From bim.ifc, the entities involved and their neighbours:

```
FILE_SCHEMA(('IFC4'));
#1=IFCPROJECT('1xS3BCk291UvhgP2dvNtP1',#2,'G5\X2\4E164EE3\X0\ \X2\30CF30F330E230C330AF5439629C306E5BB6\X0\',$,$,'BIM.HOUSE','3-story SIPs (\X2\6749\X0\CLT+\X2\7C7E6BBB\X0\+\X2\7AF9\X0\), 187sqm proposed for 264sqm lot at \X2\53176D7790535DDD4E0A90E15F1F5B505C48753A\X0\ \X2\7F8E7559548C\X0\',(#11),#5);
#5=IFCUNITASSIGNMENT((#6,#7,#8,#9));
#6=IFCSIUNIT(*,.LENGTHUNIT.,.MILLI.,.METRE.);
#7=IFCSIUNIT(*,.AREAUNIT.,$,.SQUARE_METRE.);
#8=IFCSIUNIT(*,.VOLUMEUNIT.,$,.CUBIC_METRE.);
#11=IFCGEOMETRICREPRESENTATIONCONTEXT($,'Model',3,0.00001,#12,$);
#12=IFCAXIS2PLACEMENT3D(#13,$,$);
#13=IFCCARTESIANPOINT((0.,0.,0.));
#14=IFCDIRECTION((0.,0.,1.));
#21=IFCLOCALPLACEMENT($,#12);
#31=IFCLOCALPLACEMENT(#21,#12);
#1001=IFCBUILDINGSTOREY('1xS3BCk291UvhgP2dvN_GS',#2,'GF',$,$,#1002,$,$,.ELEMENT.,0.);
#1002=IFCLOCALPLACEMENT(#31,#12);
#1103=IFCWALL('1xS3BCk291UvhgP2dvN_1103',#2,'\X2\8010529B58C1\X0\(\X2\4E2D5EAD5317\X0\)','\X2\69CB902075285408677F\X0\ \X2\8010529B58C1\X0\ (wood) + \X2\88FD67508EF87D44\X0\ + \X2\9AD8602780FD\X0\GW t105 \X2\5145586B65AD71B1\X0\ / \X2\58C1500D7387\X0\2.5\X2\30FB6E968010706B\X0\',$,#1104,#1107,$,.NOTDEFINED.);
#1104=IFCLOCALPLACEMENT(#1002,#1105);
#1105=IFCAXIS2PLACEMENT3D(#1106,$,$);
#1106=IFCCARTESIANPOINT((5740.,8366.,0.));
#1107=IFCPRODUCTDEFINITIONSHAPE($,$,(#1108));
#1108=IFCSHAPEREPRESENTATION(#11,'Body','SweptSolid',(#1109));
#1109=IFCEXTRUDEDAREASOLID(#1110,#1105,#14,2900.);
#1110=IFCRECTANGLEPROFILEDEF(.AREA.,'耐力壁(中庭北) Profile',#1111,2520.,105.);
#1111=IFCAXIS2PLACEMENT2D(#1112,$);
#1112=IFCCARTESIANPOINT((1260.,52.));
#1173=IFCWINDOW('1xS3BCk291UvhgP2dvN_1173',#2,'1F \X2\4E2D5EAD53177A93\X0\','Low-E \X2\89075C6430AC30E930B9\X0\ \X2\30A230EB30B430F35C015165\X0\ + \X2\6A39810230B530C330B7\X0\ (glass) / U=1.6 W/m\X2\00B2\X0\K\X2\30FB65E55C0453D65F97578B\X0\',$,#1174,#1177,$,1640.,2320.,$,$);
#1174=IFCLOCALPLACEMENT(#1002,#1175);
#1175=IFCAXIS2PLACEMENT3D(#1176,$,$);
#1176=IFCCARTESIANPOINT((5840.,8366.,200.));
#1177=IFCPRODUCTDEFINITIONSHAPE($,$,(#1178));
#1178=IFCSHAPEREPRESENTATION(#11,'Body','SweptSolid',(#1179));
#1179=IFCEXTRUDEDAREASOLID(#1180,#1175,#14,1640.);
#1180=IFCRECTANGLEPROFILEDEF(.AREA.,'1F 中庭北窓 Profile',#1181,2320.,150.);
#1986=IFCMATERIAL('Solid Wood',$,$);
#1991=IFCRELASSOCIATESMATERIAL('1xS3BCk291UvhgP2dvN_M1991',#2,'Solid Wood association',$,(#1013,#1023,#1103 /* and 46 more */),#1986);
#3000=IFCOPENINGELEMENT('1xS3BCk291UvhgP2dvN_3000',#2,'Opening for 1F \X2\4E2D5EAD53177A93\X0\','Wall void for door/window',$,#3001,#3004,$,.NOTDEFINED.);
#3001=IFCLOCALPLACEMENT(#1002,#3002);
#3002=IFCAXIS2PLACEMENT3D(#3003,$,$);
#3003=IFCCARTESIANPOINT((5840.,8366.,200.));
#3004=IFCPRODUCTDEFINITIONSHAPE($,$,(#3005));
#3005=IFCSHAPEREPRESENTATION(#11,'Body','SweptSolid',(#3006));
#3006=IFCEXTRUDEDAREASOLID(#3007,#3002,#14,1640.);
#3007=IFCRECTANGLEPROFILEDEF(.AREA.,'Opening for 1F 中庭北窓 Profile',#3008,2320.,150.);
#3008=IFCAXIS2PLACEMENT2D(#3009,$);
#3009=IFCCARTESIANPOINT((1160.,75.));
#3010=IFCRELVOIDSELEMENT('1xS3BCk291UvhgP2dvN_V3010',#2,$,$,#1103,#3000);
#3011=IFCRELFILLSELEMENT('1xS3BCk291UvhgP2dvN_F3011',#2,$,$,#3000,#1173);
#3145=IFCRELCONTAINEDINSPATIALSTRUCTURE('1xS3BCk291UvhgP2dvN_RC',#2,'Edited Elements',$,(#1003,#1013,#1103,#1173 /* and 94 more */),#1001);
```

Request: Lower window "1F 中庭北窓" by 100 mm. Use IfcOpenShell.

```python
import numpy as np
import ifcopenshell
import ifcopenshell.api.geometry
import ifcopenshell.util.placement
import ifcopenshell.util.unit

model = ifcopenshell.open("bim.ifc")
unit_scale = ifcopenshell.util.unit.calculate_unit_scale(model)

window = model.by_id(1173)
opening = window.FillsVoids[0].RelatingOpeningElement
dz = -0.1 / unit_scale

shift = np.array([0.0, 0.0, dz])
# The window is not placed relative to its opening, so move both.
for product in (opening, window):
    matrix = ifcopenshell.util.placement.get_local_placement(product.ObjectPlacement)
    matrix[:3, 3] += shift
    ifcopenshell.api.geometry.edit_object_placement(model, product=product, matrix=matrix, is_si=False)

print(f"moved by {dz * unit_scale:+.3f} m")

model.write("bim_rev.ifc")
```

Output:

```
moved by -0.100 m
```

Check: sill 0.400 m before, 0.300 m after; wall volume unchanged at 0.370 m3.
